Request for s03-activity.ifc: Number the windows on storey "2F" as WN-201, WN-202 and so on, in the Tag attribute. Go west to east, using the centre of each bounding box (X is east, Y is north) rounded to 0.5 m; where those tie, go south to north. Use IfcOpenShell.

First a look at what the model holds.

```python
import ifcopenshell
import ifcopenshell.util.element
import ifcopenshell.util.placement

model = ifcopenshell.open("s03-activity.ifc")
print(model.schema)
storey = next(s for s in model.by_type("IfcBuildingStorey") if s.Name == "2F")
windows = [e for e in ifcopenshell.util.element.get_decomposition(storey) if e.is_a("IfcWindow")]
for e in sorted(windows, key=lambda e: e.id()):
    origin = ifcopenshell.util.placement.get_local_placement(e.ObjectPlacement)[:3, 3]
    print(e.id(), e.Tag, e.Name, origin.round(2) + 0.0, sep=" | ")
```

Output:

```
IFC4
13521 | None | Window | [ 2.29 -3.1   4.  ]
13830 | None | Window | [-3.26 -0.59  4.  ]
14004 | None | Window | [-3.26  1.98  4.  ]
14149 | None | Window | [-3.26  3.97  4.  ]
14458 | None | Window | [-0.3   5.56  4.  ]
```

```python
import ifcopenshell
import ifcopenshell.geom
import ifcopenshell.util.element
import ifcopenshell.util.shape

model = ifcopenshell.open("s03-activity.ifc")
settings = ifcopenshell.geom.settings()
settings.set("use-world-coords", True)


def centre(element):
    shape = ifcopenshell.geom.create_shape(settings, element)
    return ifcopenshell.util.shape.get_bbox_centroid(shape.geometry)


storey = next(s for s in model.by_type("IfcBuildingStorey") if s.Name == "2F")
windows = [e for e in ifcopenshell.util.element.get_decomposition(storey) if e.is_a("IfcWindow")]

# Insertion points can sit at a corner or the storey origin, so sort by the geometry (in metres).
centres = {e: centre(e) for e in windows}
windows.sort(key=lambda e: (round(centres[e][0] / 0.5), centres[e][1]))

for i, e in enumerate(windows, start=1):
    number = f"WN-2{i:02d}"
    e.Tag = number
    print(e.id(), number)

model.write("s03-activity_edited.ifc")
```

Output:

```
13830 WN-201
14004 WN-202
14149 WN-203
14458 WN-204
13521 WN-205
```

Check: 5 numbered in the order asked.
